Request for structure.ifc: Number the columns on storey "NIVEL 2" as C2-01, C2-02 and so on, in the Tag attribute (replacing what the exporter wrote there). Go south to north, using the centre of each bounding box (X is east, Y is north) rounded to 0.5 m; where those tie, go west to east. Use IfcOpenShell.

First a look at what the model holds.

```python
import ifcopenshell
import ifcopenshell.util.element
import ifcopenshell.util.placement

model = ifcopenshell.open("structure.ifc")
print(model.schema)
storey = next(s for s in model.by_type("IfcBuildingStorey") if s.Name == "NIVEL 2")
columns = [e for e in ifcopenshell.util.element.get_decomposition(storey) if e.is_a("IfcColumn")]
for e in sorted(columns, key=lambda e: e.id()):
    origin = ifcopenshell.util.placement.get_local_placement(e.ObjectPlacement)[:3, 3]
    print(e.id(), e.Tag, e.Name, origin.round(2) + 0.0, sep=" | ")
```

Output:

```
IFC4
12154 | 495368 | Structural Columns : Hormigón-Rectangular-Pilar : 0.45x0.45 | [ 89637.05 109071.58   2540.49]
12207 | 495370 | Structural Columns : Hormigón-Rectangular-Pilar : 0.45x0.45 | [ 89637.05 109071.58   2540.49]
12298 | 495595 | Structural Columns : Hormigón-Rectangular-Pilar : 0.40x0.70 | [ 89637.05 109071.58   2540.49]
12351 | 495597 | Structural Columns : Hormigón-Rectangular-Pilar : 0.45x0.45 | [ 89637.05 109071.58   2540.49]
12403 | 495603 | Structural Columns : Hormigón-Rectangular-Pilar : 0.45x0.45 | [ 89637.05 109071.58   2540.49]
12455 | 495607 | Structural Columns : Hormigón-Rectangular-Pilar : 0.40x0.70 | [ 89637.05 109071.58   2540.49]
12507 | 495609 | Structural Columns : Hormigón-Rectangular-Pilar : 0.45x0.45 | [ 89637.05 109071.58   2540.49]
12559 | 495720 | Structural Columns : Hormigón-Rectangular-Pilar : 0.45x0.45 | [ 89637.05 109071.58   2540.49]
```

```python
import ifcopenshell
import ifcopenshell.geom
import ifcopenshell.util.element
import ifcopenshell.util.shape

model = ifcopenshell.open("structure.ifc")
settings = ifcopenshell.geom.settings()
settings.set("use-world-coords", True)


def centre(element):
    shape = ifcopenshell.geom.create_shape(settings, element)
    return ifcopenshell.util.shape.get_bbox_centroid(shape.geometry)


storey = next(s for s in model.by_type("IfcBuildingStorey") if s.Name == "NIVEL 2")
columns = [e for e in ifcopenshell.util.element.get_decomposition(storey) if e.is_a("IfcColumn")]

# Insertion points can sit at a corner or the storey origin, so sort by the geometry (in metres).
centres = {e: centre(e) for e in columns}
columns.sort(key=lambda e: (round(centres[e][1] / 0.5), centres[e][0]))

for i, e in enumerate(columns, start=1):
    number = f"C2-{i:02d}"
    e.Tag = number
    print(e.id(), number)

model.write("structure_edited.ifc")
```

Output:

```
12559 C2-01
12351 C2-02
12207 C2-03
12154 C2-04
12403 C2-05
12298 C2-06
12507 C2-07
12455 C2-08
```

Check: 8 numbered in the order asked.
